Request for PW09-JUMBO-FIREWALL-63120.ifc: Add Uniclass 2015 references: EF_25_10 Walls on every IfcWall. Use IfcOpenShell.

First a look at what the model holds.

```python
import ifcopenshell

model = ifcopenshell.open("PW09-JUMBO-FIREWALL-63120.ifc")
print(model.schema)
print("classifications:", [c.Name for c in model.by_type("IfcClassification")])
for ifc_class in ("IfcDoor", "IfcRoof", "IfcStair", "IfcWall", "IfcWindow"):
    print(ifc_class, len(model.by_type(ifc_class)))
```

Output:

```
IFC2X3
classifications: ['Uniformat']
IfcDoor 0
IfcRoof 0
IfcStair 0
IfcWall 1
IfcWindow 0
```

```python
import ifcopenshell
import ifcopenshell.api.classification

model = ifcopenshell.open("PW09-JUMBO-FIREWALL-63120.ifc")

# IFC2X3 requires Source and Edition and has no link from the project to the system.
system = model.create_entity("IfcClassification", Source="NBS", Edition="2015", Name="Uniclass 2015")

codes = {
    "IfcWall": ("EF_25_10", "Walls"),
}
for ifc_class, (code, name) in codes.items():
    products = model.by_type(ifc_class)
    ifcopenshell.api.classification.add_reference(
        model, products=products, classification=system, identification=code, name=name
    )
    print(code, len(products))

model.write("PW09-JUMBO-FIREWALL-63120_v2.ifc")
```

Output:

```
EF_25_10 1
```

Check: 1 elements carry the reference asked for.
